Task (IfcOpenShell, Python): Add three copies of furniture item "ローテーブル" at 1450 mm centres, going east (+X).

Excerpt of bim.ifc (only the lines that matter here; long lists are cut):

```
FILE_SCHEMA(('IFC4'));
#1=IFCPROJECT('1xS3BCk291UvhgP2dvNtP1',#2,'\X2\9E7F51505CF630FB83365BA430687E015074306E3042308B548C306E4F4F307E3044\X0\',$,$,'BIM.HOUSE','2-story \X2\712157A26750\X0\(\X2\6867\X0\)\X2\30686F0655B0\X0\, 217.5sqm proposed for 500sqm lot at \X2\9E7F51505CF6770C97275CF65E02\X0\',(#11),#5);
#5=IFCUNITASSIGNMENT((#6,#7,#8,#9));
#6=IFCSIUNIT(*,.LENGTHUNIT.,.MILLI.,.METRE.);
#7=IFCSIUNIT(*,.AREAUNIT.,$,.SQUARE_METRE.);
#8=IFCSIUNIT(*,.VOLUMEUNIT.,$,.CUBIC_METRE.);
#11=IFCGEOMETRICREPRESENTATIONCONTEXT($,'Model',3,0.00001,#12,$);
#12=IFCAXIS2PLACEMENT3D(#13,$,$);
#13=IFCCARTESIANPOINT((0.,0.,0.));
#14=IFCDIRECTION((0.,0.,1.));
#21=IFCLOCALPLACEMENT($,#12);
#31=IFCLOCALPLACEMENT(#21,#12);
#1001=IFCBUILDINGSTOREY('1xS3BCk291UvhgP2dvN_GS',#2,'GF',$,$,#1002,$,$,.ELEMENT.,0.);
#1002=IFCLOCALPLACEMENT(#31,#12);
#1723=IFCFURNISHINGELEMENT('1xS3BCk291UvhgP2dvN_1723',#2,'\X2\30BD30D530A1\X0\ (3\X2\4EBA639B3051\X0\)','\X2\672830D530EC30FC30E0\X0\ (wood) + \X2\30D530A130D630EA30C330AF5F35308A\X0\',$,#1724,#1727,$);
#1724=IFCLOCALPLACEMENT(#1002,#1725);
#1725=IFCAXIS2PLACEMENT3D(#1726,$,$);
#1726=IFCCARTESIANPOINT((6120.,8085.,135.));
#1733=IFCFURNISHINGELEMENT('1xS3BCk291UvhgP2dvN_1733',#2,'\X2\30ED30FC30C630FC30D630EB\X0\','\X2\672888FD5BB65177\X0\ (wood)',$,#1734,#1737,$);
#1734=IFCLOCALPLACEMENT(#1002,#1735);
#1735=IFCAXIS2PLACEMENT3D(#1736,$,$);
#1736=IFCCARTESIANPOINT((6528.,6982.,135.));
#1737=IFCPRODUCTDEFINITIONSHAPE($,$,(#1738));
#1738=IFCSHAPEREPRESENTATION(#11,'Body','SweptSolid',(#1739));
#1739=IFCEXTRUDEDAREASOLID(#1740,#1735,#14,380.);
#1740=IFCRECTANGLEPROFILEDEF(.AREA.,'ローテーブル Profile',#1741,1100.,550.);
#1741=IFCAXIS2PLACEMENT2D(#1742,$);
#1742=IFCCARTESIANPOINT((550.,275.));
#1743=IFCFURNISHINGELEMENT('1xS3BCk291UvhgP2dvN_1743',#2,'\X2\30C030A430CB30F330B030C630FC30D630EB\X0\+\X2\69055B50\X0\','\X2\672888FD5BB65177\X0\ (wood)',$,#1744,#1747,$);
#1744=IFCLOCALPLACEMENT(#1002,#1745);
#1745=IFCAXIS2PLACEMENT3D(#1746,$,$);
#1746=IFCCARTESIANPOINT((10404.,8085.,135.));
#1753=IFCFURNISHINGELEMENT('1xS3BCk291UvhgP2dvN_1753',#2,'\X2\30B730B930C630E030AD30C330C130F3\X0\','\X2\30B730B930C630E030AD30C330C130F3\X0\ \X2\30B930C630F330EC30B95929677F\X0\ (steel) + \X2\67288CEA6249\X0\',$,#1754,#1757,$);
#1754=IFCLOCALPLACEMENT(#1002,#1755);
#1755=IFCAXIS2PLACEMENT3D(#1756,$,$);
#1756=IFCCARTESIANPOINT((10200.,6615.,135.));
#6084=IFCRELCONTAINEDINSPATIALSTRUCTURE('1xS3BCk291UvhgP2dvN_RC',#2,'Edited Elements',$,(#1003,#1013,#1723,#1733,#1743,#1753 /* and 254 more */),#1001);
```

```python
import numpy as np
import ifcopenshell
import ifcopenshell.api.geometry
import ifcopenshell.api.root
import ifcopenshell.util.element
import ifcopenshell.util.placement

model = ifcopenshell.open("bim.ifc")


def reuse_history(source, copy):
    """copy_class also copies each property set's owner history, people and application; keep the originals."""
    for rel in copy.IsDefinedBy:
        if rel.is_a("IfcRelDefinesByProperties") and (history := rel.RelatingPropertyDefinition.OwnerHistory):
            rel.RelatingPropertyDefinition.OwnerHistory = source.OwnerHistory
            ifcopenshell.util.element.remove_deep2(model, history)


source = model.by_guid("1xS3BCk291UvhgP2dvN_1733")
base = ifcopenshell.util.placement.get_local_placement(source.ObjectPlacement)
step = np.array([1.0, 0.0, 0.0]) * 1450.0

for i in range(1, 4):
    copy = ifcopenshell.api.root.copy_class(model, product=source)
    copy.Representation = ifcopenshell.util.element.copy_deep(
        model, source.Representation, exclude=["IfcGeometricRepresentationContext", "IfcRepresentationMap"]
    )
    reuse_history(source, copy)
    matrix = base.copy()
    matrix[:3, 3] += i * step
    print("added at", matrix[:3, 3].round(3) + 0.0)
    ifcopenshell.api.geometry.edit_object_placement(model, product=copy, matrix=matrix, is_si=False)

model.write("bim_rev.ifc")
```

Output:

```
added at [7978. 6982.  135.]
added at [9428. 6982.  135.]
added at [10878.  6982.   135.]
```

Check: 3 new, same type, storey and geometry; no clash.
